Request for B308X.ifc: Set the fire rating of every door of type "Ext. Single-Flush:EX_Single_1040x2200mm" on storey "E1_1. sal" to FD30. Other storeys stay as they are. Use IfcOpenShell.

First a look at what the model holds.

```python
import ifcopenshell
import ifcopenshell.util.element

model = ifcopenshell.open("B308X.ifc")
print(model.schema)
storey = next(s for s in model.by_type("IfcBuildingStorey") if s.Name == "E1_1. sal")
doors = [e for e in ifcopenshell.util.element.get_decomposition(storey) if e.is_a("IfcDoor")]
seen = {}
for e in doors:
    element_type = ifcopenshell.util.element.get_type(e)
    key = (element_type.Name if element_type != e and element_type else None, ifcopenshell.util.element.get_pset(e, "Pset_DoorCommon", "FireRating"))
    seen[key] = seen.get(key, 0) + 1
for (name, value), count in sorted(seen.items(), key=str):
    print(count, "x", name, "|", value)
```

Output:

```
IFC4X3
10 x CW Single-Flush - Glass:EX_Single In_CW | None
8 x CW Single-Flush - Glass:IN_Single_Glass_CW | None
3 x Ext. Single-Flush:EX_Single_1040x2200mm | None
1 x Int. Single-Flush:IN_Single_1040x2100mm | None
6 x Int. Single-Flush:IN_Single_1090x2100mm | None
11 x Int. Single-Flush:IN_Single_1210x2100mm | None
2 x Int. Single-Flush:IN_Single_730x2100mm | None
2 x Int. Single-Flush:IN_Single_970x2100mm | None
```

```python
import ifcopenshell
import ifcopenshell.api.pset
import ifcopenshell.util.element

model = ifcopenshell.open("B308X.ifc")

storey = next(s for s in model.by_type("IfcBuildingStorey") if s.Name == "E1_1. sal")
doors = [e for e in ifcopenshell.util.element.get_decomposition(storey) if e.is_a("IfcDoor")]

count = 0
for e in doors:
    element_type = ifcopenshell.util.element.get_type(e)
    if element_type in (None, e) or element_type.Name != "Ext. Single-Flush:EX_Single_1040x2200mm":
        continue
    # add_pset returns the element's existing set when there is one.
    pset = ifcopenshell.api.pset.add_pset(model, product=e, name="Pset_DoorCommon")
    ifcopenshell.api.pset.edit_pset(model, pset=pset, properties={"FireRating": "FD30"})
    count += 1

print(count, "doors updated")

model.write("B308X_rev.ifc")
```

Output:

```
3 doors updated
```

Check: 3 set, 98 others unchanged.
